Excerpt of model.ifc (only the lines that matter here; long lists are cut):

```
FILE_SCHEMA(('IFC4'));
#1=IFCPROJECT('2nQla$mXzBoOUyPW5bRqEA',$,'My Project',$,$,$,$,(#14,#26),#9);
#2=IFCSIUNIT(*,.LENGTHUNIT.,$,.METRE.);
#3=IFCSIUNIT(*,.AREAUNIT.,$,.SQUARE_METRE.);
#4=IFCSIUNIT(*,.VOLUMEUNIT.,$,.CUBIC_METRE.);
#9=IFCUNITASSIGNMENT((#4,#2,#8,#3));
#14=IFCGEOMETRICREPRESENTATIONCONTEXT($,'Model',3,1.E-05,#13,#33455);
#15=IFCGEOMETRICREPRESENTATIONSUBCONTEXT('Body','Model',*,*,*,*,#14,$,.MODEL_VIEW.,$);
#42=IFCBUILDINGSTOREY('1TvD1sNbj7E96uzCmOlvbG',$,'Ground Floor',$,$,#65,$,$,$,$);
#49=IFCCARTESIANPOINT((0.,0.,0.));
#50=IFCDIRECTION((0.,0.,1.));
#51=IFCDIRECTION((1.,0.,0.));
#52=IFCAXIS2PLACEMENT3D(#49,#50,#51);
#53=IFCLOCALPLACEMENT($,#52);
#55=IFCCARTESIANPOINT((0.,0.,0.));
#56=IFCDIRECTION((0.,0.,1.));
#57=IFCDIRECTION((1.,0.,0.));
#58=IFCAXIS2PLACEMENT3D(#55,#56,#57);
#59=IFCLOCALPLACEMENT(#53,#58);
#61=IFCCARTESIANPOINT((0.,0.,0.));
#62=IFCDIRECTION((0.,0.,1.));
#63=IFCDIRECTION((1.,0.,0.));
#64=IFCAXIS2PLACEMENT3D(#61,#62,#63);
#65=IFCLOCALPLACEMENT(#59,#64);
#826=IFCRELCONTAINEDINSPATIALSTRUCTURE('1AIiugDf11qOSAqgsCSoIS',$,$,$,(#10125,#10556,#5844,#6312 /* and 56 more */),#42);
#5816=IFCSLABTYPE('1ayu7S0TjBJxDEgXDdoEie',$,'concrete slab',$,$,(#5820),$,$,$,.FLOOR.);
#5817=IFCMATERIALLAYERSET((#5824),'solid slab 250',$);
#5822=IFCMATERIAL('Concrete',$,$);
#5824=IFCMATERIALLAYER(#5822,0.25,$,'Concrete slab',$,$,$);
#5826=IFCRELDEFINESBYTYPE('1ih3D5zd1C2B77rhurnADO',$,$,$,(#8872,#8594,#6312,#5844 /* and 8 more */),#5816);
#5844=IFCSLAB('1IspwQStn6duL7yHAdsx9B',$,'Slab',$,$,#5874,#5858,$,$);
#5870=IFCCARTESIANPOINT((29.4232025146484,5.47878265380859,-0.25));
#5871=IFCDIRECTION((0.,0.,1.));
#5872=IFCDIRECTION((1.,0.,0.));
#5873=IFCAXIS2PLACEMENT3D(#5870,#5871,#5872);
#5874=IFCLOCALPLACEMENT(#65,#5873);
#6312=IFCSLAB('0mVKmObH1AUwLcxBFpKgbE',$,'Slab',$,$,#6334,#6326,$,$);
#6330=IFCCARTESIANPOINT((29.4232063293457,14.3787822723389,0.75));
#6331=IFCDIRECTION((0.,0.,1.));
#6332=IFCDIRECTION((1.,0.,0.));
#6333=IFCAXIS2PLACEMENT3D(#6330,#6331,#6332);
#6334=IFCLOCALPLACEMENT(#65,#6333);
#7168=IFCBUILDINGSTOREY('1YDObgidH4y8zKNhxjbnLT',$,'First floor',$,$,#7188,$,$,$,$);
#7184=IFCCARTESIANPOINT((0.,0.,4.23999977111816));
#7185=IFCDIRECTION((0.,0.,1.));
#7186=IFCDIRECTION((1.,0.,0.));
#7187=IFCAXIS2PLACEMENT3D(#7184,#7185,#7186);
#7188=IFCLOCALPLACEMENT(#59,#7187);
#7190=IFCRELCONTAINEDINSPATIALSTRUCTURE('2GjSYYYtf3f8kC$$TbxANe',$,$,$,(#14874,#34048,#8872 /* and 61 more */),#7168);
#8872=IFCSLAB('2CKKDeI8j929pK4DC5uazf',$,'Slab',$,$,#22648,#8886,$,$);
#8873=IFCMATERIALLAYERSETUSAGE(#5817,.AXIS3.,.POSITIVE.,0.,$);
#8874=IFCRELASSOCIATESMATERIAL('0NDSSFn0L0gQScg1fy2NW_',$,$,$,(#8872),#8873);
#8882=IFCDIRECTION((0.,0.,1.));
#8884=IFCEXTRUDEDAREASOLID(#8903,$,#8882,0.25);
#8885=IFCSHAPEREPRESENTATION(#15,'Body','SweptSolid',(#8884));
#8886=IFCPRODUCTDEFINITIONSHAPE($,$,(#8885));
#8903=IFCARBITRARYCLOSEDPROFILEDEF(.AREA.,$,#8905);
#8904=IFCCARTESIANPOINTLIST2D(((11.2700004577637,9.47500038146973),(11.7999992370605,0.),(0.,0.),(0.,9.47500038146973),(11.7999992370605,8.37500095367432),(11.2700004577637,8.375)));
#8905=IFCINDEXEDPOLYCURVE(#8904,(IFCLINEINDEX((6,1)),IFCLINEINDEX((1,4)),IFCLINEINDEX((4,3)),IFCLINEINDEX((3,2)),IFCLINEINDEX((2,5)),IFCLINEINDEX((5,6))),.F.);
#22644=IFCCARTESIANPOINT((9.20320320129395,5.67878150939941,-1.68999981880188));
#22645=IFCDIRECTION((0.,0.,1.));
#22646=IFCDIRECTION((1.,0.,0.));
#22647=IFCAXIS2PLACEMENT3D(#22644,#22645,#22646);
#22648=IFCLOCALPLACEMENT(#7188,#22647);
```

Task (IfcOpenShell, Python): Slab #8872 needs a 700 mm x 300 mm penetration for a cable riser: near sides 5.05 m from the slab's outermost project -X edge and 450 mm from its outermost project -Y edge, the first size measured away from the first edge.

```python
import numpy as np
import ifcopenshell
import ifcopenshell.api.feature
import ifcopenshell.api.geometry
import ifcopenshell.api.root
import ifcopenshell.geom
import ifcopenshell.util.placement
import ifcopenshell.util.representation
import ifcopenshell.util.shape
import ifcopenshell.util.unit

model = ifcopenshell.open("model.ifc")
unit_scale = ifcopenshell.util.unit.calculate_unit_scale(model)
settings = ifcopenshell.geom.settings()


def volume(element):
    """Net volume in cubic metres, openings subtracted."""
    shape = ifcopenshell.geom.create_shape(settings, element)
    return ifcopenshell.util.shape.get_volume(shape.geometry)


slab = model.by_id(8872)
before = volume(slab)

# Extent in the slab's own axes, in metres. The edges named are its -X and -Y sides.
slab_shape = ifcopenshell.geom.create_shape(settings, slab)
vertices = ifcopenshell.util.shape.get_vertices(slab_shape.geometry)
x_min, y_min, bottom = vertices.min(axis=0)
top = vertices[:, 2].max()

opening = ifcopenshell.api.root.create_entity(model, ifc_class="IfcOpeningElement", name="Cable riser opening", predefined_type="OPENING")
context = ifcopenshell.util.representation.get_context(model, "Model", "Body", "MODEL_VIEW")
width, depth = 0.7, 0.3
outline = [(0.0, 0.0), (width, 0.0), (width, depth), (0.0, depth), (0.0, 0.0)]
# Overshoot both faces by 50 mm so the cut is clean.
shape = ifcopenshell.api.geometry.add_slab_representation(
    model, context=context, depth=top - bottom + 0.1, polyline=outline
)
ifcopenshell.api.geometry.assign_representation(model, product=opening, representation=shape)

matrix = ifcopenshell.util.placement.get_local_placement(slab.ObjectPlacement)
matrix[:, 3] = matrix @ np.append(np.array([x_min + 5.05, y_min + 0.45, bottom - 0.05]) / unit_scale, 1.0)
ifcopenshell.api.geometry.edit_object_placement(model, product=opening, matrix=matrix, is_si=False)
ifcopenshell.api.feature.add_feature(model, feature=opening, element=slab)

after = volume(slab)

print(f"slab volume {before:.3f} -> {after:.3f} m3")

model.write("model_updated.ifc")
```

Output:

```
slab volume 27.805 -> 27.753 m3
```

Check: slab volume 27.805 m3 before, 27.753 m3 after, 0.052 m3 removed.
